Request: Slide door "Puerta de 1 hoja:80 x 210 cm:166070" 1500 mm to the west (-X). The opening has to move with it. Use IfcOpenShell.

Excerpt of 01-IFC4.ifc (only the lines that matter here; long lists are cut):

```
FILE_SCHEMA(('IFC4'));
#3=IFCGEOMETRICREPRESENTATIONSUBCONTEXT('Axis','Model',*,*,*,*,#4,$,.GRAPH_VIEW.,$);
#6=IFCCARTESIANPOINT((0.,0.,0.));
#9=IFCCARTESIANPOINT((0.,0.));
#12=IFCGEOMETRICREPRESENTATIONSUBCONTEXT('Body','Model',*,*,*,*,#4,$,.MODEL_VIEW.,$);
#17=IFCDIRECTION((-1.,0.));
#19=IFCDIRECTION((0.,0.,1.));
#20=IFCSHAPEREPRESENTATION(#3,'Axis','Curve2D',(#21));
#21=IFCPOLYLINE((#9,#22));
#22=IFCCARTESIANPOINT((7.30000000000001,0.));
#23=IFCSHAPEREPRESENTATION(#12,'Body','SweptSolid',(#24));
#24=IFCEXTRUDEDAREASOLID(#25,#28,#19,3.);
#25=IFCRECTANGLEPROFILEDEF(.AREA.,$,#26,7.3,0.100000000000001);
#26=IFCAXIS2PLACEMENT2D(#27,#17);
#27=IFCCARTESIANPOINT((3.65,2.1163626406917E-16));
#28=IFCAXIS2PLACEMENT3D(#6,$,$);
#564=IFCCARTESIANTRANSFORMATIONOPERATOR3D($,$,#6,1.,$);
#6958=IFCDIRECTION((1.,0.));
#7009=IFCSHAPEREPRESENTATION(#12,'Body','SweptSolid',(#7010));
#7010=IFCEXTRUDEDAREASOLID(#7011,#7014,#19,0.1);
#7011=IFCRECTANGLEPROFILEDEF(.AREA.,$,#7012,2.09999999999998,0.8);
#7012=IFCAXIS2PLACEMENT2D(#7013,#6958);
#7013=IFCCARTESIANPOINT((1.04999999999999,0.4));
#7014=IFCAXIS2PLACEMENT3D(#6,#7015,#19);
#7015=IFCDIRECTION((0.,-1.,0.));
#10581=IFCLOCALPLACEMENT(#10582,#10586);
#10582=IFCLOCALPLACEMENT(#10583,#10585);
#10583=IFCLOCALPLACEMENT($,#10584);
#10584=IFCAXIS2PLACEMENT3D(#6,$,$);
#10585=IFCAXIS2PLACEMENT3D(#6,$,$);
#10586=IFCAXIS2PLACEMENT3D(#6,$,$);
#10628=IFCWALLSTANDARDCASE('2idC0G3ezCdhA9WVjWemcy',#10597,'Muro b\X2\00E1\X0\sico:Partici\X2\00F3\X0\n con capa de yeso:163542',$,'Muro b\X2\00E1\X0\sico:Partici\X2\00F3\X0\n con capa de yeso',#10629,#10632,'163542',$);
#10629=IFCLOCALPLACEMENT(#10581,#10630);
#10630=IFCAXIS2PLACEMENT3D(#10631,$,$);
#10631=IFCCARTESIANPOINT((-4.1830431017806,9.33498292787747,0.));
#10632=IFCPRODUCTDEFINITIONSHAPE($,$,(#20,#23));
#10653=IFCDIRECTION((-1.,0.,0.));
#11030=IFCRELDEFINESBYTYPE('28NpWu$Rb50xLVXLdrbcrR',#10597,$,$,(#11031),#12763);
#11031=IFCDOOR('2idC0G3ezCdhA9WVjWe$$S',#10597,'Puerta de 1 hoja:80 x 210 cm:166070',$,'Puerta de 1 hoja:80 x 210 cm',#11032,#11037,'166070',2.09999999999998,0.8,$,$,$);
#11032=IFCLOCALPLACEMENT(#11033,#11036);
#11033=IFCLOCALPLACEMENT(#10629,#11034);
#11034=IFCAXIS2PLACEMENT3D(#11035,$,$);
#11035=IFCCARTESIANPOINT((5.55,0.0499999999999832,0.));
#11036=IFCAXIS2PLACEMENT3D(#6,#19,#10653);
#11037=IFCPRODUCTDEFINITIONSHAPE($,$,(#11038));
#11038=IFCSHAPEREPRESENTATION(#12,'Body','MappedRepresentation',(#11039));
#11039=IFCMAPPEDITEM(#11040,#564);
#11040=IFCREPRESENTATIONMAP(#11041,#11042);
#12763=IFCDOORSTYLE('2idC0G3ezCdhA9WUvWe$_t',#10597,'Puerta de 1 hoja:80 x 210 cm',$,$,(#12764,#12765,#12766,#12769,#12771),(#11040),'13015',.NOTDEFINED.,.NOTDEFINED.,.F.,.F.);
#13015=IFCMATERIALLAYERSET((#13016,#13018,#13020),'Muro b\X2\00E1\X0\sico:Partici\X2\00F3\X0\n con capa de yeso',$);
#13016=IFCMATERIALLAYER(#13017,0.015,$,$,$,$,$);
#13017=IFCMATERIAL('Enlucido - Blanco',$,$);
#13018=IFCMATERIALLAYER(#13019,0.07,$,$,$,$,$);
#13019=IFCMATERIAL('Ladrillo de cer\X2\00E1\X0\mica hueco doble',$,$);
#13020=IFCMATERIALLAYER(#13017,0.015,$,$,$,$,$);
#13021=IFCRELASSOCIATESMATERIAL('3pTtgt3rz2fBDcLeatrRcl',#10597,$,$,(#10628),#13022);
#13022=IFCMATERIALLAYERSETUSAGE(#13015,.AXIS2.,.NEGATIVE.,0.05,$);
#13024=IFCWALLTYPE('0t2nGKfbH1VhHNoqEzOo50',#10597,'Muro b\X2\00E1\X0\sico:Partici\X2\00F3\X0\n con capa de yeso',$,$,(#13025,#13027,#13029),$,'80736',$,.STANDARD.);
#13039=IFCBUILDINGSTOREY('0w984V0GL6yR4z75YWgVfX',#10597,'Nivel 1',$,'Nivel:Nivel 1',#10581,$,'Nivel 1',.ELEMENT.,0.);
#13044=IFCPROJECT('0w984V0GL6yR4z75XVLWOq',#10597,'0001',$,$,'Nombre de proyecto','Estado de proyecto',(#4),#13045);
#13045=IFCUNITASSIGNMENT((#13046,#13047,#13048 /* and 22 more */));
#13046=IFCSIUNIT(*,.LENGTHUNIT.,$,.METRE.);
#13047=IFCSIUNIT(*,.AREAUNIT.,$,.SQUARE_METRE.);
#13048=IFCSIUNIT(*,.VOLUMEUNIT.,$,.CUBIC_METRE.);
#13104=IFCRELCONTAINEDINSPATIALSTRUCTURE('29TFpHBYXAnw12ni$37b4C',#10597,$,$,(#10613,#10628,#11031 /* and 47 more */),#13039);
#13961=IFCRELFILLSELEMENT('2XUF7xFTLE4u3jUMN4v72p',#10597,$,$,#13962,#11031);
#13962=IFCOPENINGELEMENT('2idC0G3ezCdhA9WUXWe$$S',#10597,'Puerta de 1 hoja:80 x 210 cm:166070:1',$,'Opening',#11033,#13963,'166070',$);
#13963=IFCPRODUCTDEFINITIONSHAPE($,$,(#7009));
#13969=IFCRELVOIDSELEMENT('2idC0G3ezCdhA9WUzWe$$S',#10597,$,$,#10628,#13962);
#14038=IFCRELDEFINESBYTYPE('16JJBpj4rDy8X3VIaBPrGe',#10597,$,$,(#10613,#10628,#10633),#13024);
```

```python
import ifcopenshell
import ifcopenshell.api.geometry
import ifcopenshell.util.placement
import ifcopenshell.util.unit

model = ifcopenshell.open("01-IFC4.ifc")
unit_scale = ifcopenshell.util.unit.calculate_unit_scale(model)

door = model.by_guid("2idC0G3ezCdhA9WVjWe$$S")
opening = door.FillsVoids[0].RelatingOpeningElement
wall = opening.VoidsElements[0].RelatingBuildingElement

wall_matrix = ifcopenshell.util.placement.get_local_placement(wall.ObjectPlacement)
shift = wall_matrix[:3, 0] * -1.5 / unit_scale
before = ifcopenshell.util.placement.get_local_placement(door.ObjectPlacement)[:3, 3].copy()

# The door is placed relative to its opening, so it follows when the opening moves.
matrix = ifcopenshell.util.placement.get_local_placement(opening.ObjectPlacement)
matrix[:3, 3] += shift
ifcopenshell.api.geometry.edit_object_placement(
    model, product=opening, matrix=matrix, is_si=False, should_transform_children=True
)

after = ifcopenshell.util.placement.get_local_placement(door.ObjectPlacement)[:3, 3]
print("door moved by", (after - before).round(3) + 0.0)

model.write("01-IFC4_v2.ifc")
```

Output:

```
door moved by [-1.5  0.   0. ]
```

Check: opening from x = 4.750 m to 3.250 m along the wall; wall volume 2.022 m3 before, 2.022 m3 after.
